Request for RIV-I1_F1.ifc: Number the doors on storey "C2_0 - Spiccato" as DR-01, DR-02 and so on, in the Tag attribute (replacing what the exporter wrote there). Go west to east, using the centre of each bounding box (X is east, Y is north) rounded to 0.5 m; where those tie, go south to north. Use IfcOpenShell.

First a look at what the model holds.

```python
import ifcopenshell
import ifcopenshell.util.element
import ifcopenshell.util.placement

model = ifcopenshell.open("RIV-I1_F1.ifc")
print(model.schema)
storey = next(s for s in model.by_type("IfcBuildingStorey") if s.Name == "C2_0 - Spiccato")
doors = [e for e in ifcopenshell.util.element.get_decomposition(storey) if e.is_a("IfcDoor")]
for e in sorted(doors, key=lambda e: e.id()):
    origin = ifcopenshell.util.placement.get_local_placement(e.ObjectPlacement)[:3, 3]
    print(e.id(), e.Tag, e.Name, origin.round(2) + 0.0, sep=" | ")
```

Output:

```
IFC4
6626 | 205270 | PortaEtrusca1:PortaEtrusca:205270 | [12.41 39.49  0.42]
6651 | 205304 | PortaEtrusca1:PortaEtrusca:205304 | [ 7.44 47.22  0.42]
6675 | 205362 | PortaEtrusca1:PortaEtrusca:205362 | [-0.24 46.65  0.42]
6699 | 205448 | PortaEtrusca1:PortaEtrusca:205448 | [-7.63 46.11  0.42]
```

```python
import ifcopenshell
import ifcopenshell.geom
import ifcopenshell.util.element
import ifcopenshell.util.shape

model = ifcopenshell.open("RIV-I1_F1.ifc")
settings = ifcopenshell.geom.settings()
settings.set("use-world-coords", True)


def centre(element):
    shape = ifcopenshell.geom.create_shape(settings, element)
    return ifcopenshell.util.shape.get_bbox_centroid(shape.geometry)


storey = next(s for s in model.by_type("IfcBuildingStorey") if s.Name == "C2_0 - Spiccato")
doors = [e for e in ifcopenshell.util.element.get_decomposition(storey) if e.is_a("IfcDoor")]

# Insertion points can sit at a corner or the storey origin, so sort by the geometry (in metres).
centres = {e: centre(e) for e in doors}
doors.sort(key=lambda e: (round(centres[e][0] / 0.5), centres[e][1]))

for i, e in enumerate(doors, start=1):
    number = f"DR-{i:02d}"
    e.Tag = number
    print(e.id(), number)

model.write("RIV-I1_F1-out.ifc")
```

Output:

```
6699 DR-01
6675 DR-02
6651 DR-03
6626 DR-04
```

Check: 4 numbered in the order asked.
